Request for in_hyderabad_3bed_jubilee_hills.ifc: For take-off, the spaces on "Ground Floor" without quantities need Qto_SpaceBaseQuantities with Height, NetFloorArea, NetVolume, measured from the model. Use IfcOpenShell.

First a look at what the model holds.

```python
import ifcopenshell
import ifcopenshell.util.element
import ifcopenshell.util.unit

model = ifcopenshell.open("in_hyderabad_3bed_jubilee_hills.ifc")
print(model.schema)
for unit_type in ("LENGTHUNIT", "AREAUNIT", "VOLUMEUNIT"):
    print(unit_type, ifcopenshell.util.unit.calculate_unit_scale(model, unit_type))
storey = next(s for s in model.by_type("IfcBuildingStorey") if s.Name == "Ground Floor")
spaces = [e for e in ifcopenshell.util.element.get_decomposition(storey) if e.is_a("IfcSpace")]
for e in sorted(spaces, key=lambda e: e.id()):
    print(e.id(), e.is_a(), e.Name, list(ifcopenshell.util.element.get_psets(e, qtos_only=True)), sep=" | ")
```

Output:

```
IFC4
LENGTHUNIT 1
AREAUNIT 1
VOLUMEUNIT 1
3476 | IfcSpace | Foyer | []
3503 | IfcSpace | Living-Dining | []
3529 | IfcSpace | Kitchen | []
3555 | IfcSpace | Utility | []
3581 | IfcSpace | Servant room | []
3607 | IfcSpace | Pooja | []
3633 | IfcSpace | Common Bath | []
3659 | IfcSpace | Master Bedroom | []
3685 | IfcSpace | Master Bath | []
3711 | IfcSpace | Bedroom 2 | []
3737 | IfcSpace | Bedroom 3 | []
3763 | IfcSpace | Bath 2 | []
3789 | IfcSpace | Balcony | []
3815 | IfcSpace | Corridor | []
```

```python
import ifcopenshell
import ifcopenshell.api.pset
import ifcopenshell.geom
import ifcopenshell.util.element
import ifcopenshell.util.shape
import ifcopenshell.util.unit

model = ifcopenshell.open("in_hyderabad_3bed_jubilee_hills.ifc")
unit_scale = ifcopenshell.util.unit.calculate_unit_scale(model)
area_scale = ifcopenshell.util.unit.calculate_unit_scale(model, "AREAUNIT")
volume_scale = ifcopenshell.util.unit.calculate_unit_scale(model, "VOLUMEUNIT")
settings = ifcopenshell.geom.settings()

storey = next(s for s in model.by_type("IfcBuildingStorey") if s.Name == "Ground Floor")
spaces = [e for e in ifcopenshell.util.element.get_decomposition(storey) if e.is_a("IfcSpace")]

for e in sorted(spaces, key=lambda e: e.id()):
    if ifcopenshell.util.element.get_psets(e, qtos_only=True, should_inherit=False):
        continue
    # Geometry comes back in metres, in the element's own axes.
    shape = ifcopenshell.geom.create_shape(settings, e)
    values = {
        "Height": ifcopenshell.util.shape.get_z(shape.geometry) / unit_scale,
        "NetFloorArea": ifcopenshell.util.shape.get_footprint_area(shape.geometry) / area_scale,
        "NetVolume": ifcopenshell.util.shape.get_volume(shape.geometry) / volume_scale,
    }
    qto = ifcopenshell.api.pset.add_qto(model, product=e, name="Qto_SpaceBaseQuantities")
    ifcopenshell.api.pset.edit_qto(model, qto=qto, properties=values)
    print(e.id(), {k: round(v, 3) for k, v in values.items()})

model.write("in_hyderabad_3bed_jubilee_hills-out.ifc")
```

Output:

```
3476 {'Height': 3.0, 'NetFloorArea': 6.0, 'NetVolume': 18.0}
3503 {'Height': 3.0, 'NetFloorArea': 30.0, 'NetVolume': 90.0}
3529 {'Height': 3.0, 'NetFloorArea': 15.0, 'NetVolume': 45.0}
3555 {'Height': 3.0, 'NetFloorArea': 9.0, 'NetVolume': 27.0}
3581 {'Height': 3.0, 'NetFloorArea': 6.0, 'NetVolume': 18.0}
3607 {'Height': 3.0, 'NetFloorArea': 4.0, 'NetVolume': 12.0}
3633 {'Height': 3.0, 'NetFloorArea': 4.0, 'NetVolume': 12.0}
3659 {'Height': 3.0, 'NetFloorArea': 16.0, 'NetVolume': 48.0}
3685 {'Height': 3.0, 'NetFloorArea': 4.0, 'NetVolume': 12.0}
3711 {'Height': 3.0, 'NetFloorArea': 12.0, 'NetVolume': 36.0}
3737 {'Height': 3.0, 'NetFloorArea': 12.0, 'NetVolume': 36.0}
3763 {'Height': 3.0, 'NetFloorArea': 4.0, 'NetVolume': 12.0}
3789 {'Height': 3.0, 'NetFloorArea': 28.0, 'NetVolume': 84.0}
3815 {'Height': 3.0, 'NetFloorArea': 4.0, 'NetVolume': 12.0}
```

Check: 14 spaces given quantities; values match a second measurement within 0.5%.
